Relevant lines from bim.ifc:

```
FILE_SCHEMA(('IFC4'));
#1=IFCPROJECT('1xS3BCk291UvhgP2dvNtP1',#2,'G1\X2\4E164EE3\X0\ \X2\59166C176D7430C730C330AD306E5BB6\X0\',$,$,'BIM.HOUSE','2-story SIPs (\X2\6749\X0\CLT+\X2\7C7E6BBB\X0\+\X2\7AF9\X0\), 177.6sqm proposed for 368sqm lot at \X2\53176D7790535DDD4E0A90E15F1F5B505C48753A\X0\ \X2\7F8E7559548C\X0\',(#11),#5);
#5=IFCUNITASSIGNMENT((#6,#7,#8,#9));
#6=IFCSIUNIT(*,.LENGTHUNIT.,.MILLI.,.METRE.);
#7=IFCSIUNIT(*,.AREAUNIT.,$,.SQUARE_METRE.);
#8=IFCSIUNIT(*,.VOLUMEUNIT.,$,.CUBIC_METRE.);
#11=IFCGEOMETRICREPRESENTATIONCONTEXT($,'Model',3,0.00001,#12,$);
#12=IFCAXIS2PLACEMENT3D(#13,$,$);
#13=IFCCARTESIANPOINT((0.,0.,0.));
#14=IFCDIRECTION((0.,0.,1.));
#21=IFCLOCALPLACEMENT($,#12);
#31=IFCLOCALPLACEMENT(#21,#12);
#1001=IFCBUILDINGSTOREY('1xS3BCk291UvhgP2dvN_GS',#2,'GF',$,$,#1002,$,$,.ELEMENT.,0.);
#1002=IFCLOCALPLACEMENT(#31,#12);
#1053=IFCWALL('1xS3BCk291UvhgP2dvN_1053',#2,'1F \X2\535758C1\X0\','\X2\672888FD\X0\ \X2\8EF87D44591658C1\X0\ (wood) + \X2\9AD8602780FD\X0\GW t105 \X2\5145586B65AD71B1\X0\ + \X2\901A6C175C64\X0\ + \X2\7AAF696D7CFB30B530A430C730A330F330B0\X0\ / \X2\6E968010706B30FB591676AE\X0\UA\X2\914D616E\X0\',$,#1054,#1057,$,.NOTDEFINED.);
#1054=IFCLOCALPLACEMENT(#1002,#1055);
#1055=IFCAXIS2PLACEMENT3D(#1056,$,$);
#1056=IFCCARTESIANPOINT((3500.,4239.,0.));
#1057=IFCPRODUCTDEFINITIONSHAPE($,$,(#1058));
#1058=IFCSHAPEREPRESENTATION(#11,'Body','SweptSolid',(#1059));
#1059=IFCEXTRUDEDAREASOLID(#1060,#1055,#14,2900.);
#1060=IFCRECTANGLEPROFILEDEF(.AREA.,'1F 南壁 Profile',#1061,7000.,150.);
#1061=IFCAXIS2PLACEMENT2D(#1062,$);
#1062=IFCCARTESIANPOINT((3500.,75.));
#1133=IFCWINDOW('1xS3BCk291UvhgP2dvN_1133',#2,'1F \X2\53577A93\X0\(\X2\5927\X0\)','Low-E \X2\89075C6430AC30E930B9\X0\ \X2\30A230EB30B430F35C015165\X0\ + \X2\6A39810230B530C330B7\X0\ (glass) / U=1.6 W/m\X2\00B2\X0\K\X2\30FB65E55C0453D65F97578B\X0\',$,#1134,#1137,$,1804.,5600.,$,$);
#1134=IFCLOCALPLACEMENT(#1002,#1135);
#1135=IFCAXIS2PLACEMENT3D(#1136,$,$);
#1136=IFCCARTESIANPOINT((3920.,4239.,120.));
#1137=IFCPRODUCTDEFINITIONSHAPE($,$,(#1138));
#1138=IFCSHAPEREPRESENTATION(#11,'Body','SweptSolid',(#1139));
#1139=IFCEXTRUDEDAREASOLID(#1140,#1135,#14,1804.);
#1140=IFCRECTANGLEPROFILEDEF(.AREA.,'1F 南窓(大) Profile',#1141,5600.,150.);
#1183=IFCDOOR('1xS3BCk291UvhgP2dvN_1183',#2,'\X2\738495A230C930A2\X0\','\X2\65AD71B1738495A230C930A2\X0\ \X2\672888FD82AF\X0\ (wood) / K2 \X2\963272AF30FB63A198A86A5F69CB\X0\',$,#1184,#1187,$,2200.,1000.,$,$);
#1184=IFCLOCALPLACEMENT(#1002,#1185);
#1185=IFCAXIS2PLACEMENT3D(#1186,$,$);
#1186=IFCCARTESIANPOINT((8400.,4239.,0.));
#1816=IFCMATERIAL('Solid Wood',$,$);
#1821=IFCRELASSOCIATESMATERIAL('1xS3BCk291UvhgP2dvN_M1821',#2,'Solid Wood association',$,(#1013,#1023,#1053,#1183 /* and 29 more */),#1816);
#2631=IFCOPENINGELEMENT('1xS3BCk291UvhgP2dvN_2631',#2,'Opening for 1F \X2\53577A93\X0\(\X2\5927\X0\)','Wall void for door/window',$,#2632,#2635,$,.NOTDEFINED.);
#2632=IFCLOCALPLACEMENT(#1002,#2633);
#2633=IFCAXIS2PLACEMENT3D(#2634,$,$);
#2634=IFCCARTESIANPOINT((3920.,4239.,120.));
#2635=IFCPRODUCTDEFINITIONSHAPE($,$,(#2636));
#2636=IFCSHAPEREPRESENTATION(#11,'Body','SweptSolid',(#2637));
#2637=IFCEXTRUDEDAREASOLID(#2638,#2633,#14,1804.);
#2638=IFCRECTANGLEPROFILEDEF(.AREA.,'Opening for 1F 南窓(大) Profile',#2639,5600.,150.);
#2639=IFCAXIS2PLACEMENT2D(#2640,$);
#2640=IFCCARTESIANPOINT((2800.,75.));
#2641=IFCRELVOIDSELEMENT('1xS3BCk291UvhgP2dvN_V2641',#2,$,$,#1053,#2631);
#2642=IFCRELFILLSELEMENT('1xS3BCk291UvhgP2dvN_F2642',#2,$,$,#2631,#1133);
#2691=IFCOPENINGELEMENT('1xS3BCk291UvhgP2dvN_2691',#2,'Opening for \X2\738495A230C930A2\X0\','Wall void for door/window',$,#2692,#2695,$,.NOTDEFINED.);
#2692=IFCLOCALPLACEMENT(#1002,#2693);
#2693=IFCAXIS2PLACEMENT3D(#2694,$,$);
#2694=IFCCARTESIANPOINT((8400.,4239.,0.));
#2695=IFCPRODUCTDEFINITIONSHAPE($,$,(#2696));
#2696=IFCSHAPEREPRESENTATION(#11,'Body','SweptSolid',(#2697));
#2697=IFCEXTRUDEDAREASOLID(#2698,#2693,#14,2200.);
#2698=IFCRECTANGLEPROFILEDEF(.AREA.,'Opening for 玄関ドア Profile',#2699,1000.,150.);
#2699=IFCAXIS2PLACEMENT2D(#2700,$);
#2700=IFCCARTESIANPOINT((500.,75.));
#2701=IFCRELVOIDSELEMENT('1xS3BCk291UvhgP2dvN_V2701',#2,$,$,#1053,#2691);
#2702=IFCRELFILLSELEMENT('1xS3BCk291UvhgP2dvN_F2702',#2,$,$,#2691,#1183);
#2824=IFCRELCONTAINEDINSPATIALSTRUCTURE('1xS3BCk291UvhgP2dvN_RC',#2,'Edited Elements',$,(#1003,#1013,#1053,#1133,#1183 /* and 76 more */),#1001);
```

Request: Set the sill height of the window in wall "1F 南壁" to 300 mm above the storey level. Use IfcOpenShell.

```python
import numpy as np
import ifcopenshell
import ifcopenshell.api.geometry
import ifcopenshell.geom
import ifcopenshell.util.element
import ifcopenshell.util.placement
import ifcopenshell.util.shape
import ifcopenshell.util.unit

model = ifcopenshell.open("bim.ifc")
unit_scale = ifcopenshell.util.unit.calculate_unit_scale(model)

window = model.by_guid("1xS3BCk291UvhgP2dvN_1133")
opening = window.FillsVoids[0].RelatingOpeningElement
storey = ifcopenshell.util.element.get_container(window, ifc_class="IfcBuildingStorey")
level = ifcopenshell.util.placement.get_local_placement(storey.ObjectPlacement)[2, 3]

# The opening's origin need not be at the sill, so measure its lowest point.
shape = ifcopenshell.geom.create_shape(ifcopenshell.geom.settings(), opening)
bottom = ifcopenshell.util.shape.get_shape_bottom_elevation(shape, shape.geometry) / unit_scale
dz = level + 0.3 / unit_scale - bottom

shift = np.array([0.0, 0.0, dz])
# The window is not placed relative to its opening, so move both.
for product in (opening, window):
    matrix = ifcopenshell.util.placement.get_local_placement(product.ObjectPlacement)
    matrix[:3, 3] += shift
    ifcopenshell.api.geometry.edit_object_placement(model, product=product, matrix=matrix, is_si=False)

print(f"moved by {dz * unit_scale:+.3f} m")

model.write("bim_v2.ifc")
```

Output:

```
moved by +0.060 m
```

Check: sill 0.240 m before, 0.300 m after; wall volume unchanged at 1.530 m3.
